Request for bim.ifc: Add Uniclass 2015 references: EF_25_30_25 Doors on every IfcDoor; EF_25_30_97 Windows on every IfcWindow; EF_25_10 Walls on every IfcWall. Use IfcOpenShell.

First a look at what the model holds.

```python
import ifcopenshell

model = ifcopenshell.open("bim.ifc")
print(model.schema)
print("classifications:", [c.Name for c in model.by_type("IfcClassification")])
for ifc_class in ("IfcDoor", "IfcRoof", "IfcStair", "IfcWall", "IfcWindow"):
    print(ifc_class, len(model.by_type(ifc_class)))
```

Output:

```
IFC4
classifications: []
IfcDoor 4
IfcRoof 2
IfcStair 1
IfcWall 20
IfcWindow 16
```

```python
import ifcopenshell
import ifcopenshell.api.classification

model = ifcopenshell.open("bim.ifc")

system = ifcopenshell.api.classification.add_classification(model, classification="Uniclass 2015")

codes = {
    "IfcDoor": ("EF_25_30_25", "Doors"),
    "IfcWindow": ("EF_25_30_97", "Windows"),
    "IfcWall": ("EF_25_10", "Walls"),
}
for ifc_class, (code, name) in codes.items():
    products = model.by_type(ifc_class)
    ifcopenshell.api.classification.add_reference(
        model, products=products, classification=system, identification=code, name=name
    )
    print(code, len(products))

model.write("bim_edited.ifc")
```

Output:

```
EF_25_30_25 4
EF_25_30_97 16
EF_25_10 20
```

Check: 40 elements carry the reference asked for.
